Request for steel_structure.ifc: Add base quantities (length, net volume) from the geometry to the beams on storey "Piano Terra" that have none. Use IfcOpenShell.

First a look at what the model holds.

```python
import ifcopenshell
import ifcopenshell.util.element
import ifcopenshell.util.unit

model = ifcopenshell.open("steel_structure.ifc")
print(model.schema)
for unit_type in ("LENGTHUNIT", "AREAUNIT", "VOLUMEUNIT"):
    print(unit_type, ifcopenshell.util.unit.calculate_unit_scale(model, unit_type))
storey = next(s for s in model.by_type("IfcBuildingStorey") if s.Name == "Piano Terra")
beams = [e for e in ifcopenshell.util.element.get_decomposition(storey) if e.is_a("IfcBeam")]
for e in sorted(beams, key=lambda e: e.id()):
    print(e.id(), e.is_a(), e.Name, list(ifcopenshell.util.element.get_psets(e, qtos_only=True)), sep=" | ")
```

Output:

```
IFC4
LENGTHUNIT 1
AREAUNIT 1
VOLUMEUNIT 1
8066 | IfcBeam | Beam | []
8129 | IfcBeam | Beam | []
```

```python
import ifcopenshell
import ifcopenshell.api.pset
import ifcopenshell.geom
import ifcopenshell.util.element
import ifcopenshell.util.shape
import ifcopenshell.util.unit

model = ifcopenshell.open("steel_structure.ifc")
unit_scale = ifcopenshell.util.unit.calculate_unit_scale(model)
volume_scale = ifcopenshell.util.unit.calculate_unit_scale(model, "VOLUMEUNIT")
settings = ifcopenshell.geom.settings()

storey = next(s for s in model.by_type("IfcBuildingStorey") if s.Name == "Piano Terra")
beams = [e for e in ifcopenshell.util.element.get_decomposition(storey) if e.is_a("IfcBeam")]

for e in sorted(beams, key=lambda e: e.id()):
    if ifcopenshell.util.element.get_psets(e, qtos_only=True, should_inherit=False):
        continue
    # Geometry comes back in metres, in the element's own axes.
    shape = ifcopenshell.geom.create_shape(settings, e)
    values = {
        "Length": ifcopenshell.util.shape.get_max_xyz(shape.geometry) / unit_scale,
        "NetVolume": ifcopenshell.util.shape.get_volume(shape.geometry) / volume_scale,
    }
    qto = ifcopenshell.api.pset.add_qto(model, product=e, name="Qto_BeamBaseQuantities")
    ifcopenshell.api.pset.edit_qto(model, qto=qto, properties=values)
    print(e.id(), {k: round(v, 3) for k, v in values.items()})

model.write("steel_structure_updated.ifc")
```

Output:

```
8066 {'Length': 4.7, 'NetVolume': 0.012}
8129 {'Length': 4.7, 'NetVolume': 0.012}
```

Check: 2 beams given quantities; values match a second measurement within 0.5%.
